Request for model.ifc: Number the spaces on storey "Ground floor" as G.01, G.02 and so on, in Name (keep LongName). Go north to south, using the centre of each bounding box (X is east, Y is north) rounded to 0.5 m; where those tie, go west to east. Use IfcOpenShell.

First a look at what the model holds.

```python
import ifcopenshell
import ifcopenshell.util.element
import ifcopenshell.util.placement

model = ifcopenshell.open("model.ifc")
print(model.schema)
storey = next(s for s in model.by_type("IfcBuildingStorey") if s.Name == "Ground floor")
spaces = [e for e in ifcopenshell.util.element.get_decomposition(storey) if e.is_a("IfcSpace")]
for e in sorted(spaces, key=lambda e: e.id()):
    origin = ifcopenshell.util.placement.get_local_placement(e.ObjectPlacement)[:3, 3]
    print(e.id(), e.Name, e.LongName, origin.round(2) + 0.0, sep=" | ")
```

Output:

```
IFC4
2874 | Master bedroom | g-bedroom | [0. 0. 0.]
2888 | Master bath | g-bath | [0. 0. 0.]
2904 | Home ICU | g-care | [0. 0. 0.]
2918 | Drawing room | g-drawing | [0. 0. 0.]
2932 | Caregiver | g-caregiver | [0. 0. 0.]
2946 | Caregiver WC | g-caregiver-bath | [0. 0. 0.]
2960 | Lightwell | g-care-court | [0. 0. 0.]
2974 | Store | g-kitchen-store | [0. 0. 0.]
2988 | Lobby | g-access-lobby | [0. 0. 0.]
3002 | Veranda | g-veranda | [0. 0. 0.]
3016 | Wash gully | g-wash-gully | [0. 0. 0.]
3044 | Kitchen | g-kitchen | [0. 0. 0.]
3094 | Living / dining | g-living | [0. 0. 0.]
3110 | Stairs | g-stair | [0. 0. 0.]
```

```python
import ifcopenshell
import ifcopenshell.geom
import ifcopenshell.util.element
import ifcopenshell.util.shape

model = ifcopenshell.open("model.ifc")
settings = ifcopenshell.geom.settings()
settings.set("use-world-coords", True)


def centre(element):
    shape = ifcopenshell.geom.create_shape(settings, element)
    return ifcopenshell.util.shape.get_bbox_centroid(shape.geometry)


storey = next(s for s in model.by_type("IfcBuildingStorey") if s.Name == "Ground floor")
spaces = [e for e in ifcopenshell.util.element.get_decomposition(storey) if e.is_a("IfcSpace")]

# Insertion points can sit at a corner or the storey origin, so sort by the geometry (in metres).
centres = {e: centre(e) for e in spaces}
spaces.sort(key=lambda e: (-round(centres[e][1] / 0.5), centres[e][0]))

for i, e in enumerate(spaces, start=1):
    number = f"G.{i:02d}"
    e.Name = number
    print(e.id(), number)

model.write("model_edited.ifc")
```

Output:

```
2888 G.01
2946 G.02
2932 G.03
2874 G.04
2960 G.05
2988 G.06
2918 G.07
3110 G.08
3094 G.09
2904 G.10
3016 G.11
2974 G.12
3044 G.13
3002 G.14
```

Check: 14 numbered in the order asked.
